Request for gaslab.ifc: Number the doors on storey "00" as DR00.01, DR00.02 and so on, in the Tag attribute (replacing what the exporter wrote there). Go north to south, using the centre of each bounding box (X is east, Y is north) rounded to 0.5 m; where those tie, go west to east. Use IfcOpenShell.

First a look at what the model holds.

```python
import ifcopenshell
import ifcopenshell.util.element
import ifcopenshell.util.placement

model = ifcopenshell.open("gaslab.ifc")
print(model.schema)
storey = next(s for s in model.by_type("IfcBuildingStorey") if s.Name == "00")
doors = [e for e in ifcopenshell.util.element.get_decomposition(storey) if e.is_a("IfcDoor")]
for e in sorted(doors, key=lambda e: e.id()):
    origin = ifcopenshell.util.placement.get_local_placement(e.ObjectPlacement)[:3, 3]
    print(e.id(), e.Tag, e.Name, origin.round(2) + 0.0, sep=" | ")
```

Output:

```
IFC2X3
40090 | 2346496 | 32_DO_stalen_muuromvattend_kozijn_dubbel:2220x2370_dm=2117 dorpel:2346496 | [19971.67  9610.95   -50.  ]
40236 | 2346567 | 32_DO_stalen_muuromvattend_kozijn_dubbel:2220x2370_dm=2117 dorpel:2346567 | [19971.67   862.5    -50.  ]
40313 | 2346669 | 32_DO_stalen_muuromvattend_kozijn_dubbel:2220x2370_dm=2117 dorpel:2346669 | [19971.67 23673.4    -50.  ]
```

```python
import ifcopenshell
import ifcopenshell.geom
import ifcopenshell.util.element
import ifcopenshell.util.shape

model = ifcopenshell.open("gaslab.ifc")
settings = ifcopenshell.geom.settings()
settings.set("use-world-coords", True)


def centre(element):
    shape = ifcopenshell.geom.create_shape(settings, element)
    return ifcopenshell.util.shape.get_bbox_centroid(shape.geometry)


storey = next(s for s in model.by_type("IfcBuildingStorey") if s.Name == "00")
doors = [e for e in ifcopenshell.util.element.get_decomposition(storey) if e.is_a("IfcDoor")]

# Insertion points can sit at a corner or the storey origin, so sort by the geometry (in metres).
centres = {e: centre(e) for e in doors}
doors.sort(key=lambda e: (-round(centres[e][1] / 0.5), centres[e][0]))

for i, e in enumerate(doors, start=1):
    number = f"DR00.{i:02d}"
    e.Tag = number
    print(e.id(), number)

model.write("gaslab_edited.ifc")
```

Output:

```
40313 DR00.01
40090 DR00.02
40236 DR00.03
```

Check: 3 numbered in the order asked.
